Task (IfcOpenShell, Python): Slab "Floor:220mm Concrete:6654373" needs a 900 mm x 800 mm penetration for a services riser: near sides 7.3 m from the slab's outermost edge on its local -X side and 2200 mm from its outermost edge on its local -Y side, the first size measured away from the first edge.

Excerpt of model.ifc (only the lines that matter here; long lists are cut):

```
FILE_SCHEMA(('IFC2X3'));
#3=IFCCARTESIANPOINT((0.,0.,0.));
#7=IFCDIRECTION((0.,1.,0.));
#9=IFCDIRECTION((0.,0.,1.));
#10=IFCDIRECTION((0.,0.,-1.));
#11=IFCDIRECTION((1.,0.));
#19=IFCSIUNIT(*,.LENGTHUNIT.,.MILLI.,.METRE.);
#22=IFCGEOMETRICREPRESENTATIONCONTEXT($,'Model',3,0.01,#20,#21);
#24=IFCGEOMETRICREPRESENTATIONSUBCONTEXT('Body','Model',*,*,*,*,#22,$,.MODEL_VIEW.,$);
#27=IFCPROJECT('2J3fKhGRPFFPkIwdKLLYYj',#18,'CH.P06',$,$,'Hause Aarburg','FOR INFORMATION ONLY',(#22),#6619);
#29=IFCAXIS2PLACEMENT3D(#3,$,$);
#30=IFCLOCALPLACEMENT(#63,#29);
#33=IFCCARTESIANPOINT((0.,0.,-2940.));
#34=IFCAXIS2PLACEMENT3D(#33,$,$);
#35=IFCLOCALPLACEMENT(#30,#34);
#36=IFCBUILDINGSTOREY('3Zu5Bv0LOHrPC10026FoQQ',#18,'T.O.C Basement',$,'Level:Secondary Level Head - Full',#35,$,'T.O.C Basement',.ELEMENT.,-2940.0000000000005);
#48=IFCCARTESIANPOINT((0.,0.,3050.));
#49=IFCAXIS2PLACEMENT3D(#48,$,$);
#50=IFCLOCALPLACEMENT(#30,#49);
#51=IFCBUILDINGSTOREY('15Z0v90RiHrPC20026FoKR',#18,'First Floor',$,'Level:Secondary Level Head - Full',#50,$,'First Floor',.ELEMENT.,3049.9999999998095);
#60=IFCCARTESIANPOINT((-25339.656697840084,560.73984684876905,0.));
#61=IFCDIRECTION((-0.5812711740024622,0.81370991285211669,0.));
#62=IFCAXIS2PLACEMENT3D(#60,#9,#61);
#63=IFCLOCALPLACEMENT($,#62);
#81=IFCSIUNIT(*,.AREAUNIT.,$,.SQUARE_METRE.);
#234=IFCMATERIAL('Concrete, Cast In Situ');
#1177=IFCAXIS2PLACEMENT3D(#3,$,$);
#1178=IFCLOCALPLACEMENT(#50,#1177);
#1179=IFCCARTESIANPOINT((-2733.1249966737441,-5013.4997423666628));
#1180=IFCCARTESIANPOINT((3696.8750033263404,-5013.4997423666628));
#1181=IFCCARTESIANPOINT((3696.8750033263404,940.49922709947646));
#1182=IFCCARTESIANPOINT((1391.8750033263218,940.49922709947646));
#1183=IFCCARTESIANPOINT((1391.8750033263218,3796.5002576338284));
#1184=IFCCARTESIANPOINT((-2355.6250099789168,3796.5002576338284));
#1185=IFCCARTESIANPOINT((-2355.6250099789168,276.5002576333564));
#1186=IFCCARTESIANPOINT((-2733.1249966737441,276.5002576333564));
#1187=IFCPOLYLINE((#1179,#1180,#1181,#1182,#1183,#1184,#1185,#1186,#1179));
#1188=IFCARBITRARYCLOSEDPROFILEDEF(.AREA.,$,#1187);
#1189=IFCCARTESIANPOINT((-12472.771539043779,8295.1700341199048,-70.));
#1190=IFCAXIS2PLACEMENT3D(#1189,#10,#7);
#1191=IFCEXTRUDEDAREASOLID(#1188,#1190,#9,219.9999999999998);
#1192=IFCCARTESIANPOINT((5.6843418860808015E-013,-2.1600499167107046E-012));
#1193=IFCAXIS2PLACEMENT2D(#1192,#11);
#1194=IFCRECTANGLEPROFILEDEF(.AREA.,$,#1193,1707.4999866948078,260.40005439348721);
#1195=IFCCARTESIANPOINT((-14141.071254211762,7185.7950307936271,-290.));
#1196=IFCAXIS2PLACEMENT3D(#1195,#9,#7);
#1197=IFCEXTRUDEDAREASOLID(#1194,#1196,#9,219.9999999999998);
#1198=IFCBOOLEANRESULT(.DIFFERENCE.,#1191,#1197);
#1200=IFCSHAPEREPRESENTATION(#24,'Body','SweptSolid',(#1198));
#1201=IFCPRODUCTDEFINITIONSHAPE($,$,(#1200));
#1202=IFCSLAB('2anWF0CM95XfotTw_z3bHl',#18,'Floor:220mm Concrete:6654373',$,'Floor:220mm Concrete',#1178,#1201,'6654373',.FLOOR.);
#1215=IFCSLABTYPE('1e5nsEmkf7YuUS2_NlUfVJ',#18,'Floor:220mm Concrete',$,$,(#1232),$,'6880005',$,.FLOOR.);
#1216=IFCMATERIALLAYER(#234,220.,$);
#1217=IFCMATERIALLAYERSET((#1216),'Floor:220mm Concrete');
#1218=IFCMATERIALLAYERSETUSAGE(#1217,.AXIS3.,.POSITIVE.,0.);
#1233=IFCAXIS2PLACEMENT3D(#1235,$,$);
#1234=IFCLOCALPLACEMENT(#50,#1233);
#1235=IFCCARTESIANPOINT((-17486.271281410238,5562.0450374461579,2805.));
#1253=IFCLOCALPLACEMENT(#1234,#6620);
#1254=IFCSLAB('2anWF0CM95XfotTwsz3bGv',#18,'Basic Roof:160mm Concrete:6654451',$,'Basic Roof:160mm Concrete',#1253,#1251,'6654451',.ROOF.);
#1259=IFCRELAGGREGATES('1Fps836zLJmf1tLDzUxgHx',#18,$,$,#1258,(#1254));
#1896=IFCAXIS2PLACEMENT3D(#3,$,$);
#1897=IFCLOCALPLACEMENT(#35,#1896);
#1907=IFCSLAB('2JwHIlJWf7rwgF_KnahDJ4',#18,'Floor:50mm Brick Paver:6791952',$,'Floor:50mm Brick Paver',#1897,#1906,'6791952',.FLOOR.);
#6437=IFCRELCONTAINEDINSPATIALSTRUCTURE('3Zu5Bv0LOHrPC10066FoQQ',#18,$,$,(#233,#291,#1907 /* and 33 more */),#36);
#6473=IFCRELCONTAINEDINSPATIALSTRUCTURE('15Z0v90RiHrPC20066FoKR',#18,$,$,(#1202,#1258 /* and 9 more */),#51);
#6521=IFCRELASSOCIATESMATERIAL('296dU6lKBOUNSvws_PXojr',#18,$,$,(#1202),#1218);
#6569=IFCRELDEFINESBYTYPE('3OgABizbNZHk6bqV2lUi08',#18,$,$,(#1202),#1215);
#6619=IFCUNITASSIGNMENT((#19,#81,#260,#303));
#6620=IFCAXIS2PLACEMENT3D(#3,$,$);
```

```python
import numpy as np
import ifcopenshell
import ifcopenshell.api.feature
import ifcopenshell.api.geometry
import ifcopenshell.api.root
import ifcopenshell.geom
import ifcopenshell.util.placement
import ifcopenshell.util.representation
import ifcopenshell.util.shape
import ifcopenshell.util.unit

model = ifcopenshell.open("model.ifc")
unit_scale = ifcopenshell.util.unit.calculate_unit_scale(model)
settings = ifcopenshell.geom.settings()


def volume(element):
    """Net volume in cubic metres, openings subtracted."""
    shape = ifcopenshell.geom.create_shape(settings, element)
    return ifcopenshell.util.shape.get_volume(shape.geometry)


slab = model.by_guid("2anWF0CM95XfotTw_z3bHl")
before = volume(slab)

# Extent in the slab's own axes, in metres. The edges named are its -X and -Y sides.
slab_shape = ifcopenshell.geom.create_shape(settings, slab)
vertices = ifcopenshell.util.shape.get_vertices(slab_shape.geometry)
x_min, y_min, bottom = vertices.min(axis=0)
top = vertices[:, 2].max()

opening = ifcopenshell.api.root.create_entity(model, ifc_class="IfcOpeningElement", name="Services riser opening")
context = ifcopenshell.util.representation.get_context(model, "Model", "Body", "MODEL_VIEW")
width, depth = 0.9, 0.8
outline = [(0.0, 0.0), (width, 0.0), (width, depth), (0.0, depth), (0.0, 0.0)]
# Overshoot both faces by 50 mm so the cut is clean.
shape = ifcopenshell.api.geometry.add_slab_representation(
    model, context=context, depth=top - bottom + 0.1, polyline=outline
)
ifcopenshell.api.geometry.assign_representation(model, product=opening, representation=shape)

matrix = ifcopenshell.util.placement.get_local_placement(slab.ObjectPlacement)
matrix[:, 3] = matrix @ np.append(np.array([x_min + 7.3, y_min + 2.2, bottom - 0.05]) / unit_scale, 1.0)
ifcopenshell.api.geometry.edit_object_placement(model, product=opening, matrix=matrix, is_si=False)
ifcopenshell.api.feature.add_feature(model, feature=opening, element=slab)

after = volume(slab)

print(f"slab volume {before:.3f} -> {after:.3f} m3")

model.write("model-out.ifc")
```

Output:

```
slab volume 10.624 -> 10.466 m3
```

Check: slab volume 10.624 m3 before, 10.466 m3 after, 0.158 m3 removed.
